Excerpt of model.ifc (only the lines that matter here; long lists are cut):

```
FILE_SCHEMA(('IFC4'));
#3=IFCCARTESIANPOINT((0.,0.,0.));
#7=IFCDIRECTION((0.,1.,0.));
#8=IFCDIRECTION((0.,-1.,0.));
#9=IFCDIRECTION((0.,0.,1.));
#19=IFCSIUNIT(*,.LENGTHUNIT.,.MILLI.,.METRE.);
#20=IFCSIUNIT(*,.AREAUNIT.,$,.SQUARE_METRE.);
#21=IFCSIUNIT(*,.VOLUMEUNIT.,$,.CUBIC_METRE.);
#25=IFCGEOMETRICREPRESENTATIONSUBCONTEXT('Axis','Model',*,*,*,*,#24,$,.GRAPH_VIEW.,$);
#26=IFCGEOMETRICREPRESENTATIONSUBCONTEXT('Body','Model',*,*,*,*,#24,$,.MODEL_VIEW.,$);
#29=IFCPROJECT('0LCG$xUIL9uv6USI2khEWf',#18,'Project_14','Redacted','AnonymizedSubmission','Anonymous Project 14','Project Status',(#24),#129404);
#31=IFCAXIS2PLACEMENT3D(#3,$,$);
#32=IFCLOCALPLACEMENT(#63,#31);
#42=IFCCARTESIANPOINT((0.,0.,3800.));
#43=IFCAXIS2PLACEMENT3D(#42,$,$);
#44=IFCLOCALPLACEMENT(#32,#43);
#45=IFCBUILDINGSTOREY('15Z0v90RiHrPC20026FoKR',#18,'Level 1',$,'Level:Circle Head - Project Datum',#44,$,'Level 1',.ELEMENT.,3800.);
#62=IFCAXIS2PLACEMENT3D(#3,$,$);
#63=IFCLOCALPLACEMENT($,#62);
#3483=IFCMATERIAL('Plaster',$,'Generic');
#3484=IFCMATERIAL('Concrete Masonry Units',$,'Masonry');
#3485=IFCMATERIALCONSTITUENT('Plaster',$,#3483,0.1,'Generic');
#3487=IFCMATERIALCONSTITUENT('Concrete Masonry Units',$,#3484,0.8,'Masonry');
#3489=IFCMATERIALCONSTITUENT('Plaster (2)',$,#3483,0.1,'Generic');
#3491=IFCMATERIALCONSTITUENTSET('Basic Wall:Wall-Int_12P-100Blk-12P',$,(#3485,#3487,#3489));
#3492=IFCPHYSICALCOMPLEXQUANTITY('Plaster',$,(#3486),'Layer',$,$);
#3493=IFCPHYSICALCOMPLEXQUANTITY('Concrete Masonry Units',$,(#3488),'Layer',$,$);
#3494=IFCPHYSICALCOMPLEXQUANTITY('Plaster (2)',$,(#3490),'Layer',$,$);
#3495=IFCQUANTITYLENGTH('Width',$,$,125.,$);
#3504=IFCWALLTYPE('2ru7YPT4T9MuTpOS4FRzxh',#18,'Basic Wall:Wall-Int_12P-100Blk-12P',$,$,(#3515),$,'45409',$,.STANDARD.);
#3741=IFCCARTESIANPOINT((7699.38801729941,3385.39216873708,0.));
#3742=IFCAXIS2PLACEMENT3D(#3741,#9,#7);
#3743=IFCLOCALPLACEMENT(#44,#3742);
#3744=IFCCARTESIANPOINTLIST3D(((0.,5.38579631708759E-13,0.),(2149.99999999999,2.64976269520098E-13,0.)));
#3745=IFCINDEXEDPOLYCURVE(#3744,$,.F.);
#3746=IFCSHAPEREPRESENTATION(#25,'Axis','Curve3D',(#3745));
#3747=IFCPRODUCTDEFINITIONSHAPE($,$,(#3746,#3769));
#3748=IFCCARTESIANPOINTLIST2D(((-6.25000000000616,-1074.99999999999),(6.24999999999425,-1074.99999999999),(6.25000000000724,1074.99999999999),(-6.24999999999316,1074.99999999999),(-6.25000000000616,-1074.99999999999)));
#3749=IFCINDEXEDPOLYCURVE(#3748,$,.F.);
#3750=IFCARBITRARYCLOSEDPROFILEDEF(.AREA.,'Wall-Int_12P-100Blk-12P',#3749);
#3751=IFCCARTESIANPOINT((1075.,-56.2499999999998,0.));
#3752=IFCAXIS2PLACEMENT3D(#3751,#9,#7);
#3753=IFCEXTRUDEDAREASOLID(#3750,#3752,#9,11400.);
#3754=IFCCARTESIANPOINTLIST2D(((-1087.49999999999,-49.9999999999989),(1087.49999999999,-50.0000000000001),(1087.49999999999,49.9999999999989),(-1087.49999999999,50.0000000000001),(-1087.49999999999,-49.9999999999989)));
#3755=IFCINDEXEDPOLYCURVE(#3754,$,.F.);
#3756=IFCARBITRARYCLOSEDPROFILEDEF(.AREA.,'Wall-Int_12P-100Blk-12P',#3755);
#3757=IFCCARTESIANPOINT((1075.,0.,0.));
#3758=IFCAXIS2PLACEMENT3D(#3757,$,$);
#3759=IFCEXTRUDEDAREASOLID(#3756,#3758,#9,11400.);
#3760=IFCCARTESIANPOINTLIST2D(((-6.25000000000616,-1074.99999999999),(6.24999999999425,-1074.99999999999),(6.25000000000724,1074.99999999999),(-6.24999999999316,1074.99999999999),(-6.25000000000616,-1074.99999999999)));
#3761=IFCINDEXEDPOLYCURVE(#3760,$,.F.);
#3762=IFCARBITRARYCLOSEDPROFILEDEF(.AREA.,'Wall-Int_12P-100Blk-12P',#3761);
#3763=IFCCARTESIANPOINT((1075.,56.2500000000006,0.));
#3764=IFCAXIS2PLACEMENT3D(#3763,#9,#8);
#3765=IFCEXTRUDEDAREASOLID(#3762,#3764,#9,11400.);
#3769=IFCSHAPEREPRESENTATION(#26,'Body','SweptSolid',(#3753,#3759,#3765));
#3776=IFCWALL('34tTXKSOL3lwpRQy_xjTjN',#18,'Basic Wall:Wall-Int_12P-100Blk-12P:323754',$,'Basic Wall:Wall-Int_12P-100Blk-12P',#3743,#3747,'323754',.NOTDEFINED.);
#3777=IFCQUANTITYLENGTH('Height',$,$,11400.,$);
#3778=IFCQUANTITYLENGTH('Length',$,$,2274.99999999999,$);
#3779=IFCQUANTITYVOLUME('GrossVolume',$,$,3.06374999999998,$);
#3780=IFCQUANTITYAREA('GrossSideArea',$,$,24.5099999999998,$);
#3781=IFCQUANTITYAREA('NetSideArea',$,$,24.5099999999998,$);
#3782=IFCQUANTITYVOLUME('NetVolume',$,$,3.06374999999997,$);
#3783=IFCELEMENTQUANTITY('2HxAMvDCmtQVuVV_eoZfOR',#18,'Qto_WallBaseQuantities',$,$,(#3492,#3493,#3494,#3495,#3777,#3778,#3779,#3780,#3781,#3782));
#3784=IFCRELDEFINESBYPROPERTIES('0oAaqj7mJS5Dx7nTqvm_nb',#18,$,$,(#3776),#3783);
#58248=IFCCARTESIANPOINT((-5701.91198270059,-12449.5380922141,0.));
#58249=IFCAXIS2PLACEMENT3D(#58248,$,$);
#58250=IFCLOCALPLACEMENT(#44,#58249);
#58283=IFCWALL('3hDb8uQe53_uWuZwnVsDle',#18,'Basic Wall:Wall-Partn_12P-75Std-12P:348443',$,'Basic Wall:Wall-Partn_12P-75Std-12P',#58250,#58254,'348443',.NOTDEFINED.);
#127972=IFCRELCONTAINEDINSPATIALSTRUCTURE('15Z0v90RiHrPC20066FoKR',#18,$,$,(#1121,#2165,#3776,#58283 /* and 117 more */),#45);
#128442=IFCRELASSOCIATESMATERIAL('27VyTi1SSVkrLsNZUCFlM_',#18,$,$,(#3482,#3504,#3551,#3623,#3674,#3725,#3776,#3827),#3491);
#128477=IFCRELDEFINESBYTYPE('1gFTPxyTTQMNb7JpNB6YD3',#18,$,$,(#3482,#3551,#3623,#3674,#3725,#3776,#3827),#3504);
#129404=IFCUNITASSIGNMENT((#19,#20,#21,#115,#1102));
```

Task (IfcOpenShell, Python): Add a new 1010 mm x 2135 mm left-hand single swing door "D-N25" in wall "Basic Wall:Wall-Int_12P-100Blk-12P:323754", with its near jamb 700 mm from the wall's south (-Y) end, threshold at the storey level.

```python
import numpy as np
import ifcopenshell
import ifcopenshell.api.feature
import ifcopenshell.api.geometry
import ifcopenshell.api.pset
import ifcopenshell.api.root
import ifcopenshell.api.spatial
import ifcopenshell.geom
import ifcopenshell.util.element
import ifcopenshell.util.placement
import ifcopenshell.util.representation
import ifcopenshell.util.shape
import ifcopenshell.util.unit

model = ifcopenshell.open("model.ifc")
unit_scale = ifcopenshell.util.unit.calculate_unit_scale(model)
area_scale = ifcopenshell.util.unit.calculate_unit_scale(model, "AREAUNIT")
volume_scale = ifcopenshell.util.unit.calculate_unit_scale(model, "VOLUMEUNIT")
settings = ifcopenshell.geom.settings()


def volume(element):
    """Net volume in cubic metres, openings subtracted."""
    shape = ifcopenshell.geom.create_shape(settings, element)
    return ifcopenshell.util.shape.get_volume(shape.geometry)


wall = model.by_guid("34tTXKSOL3lwpRQy_xjTjN")
storey = ifcopenshell.util.element.get_container(wall, ifc_class="IfcBuildingStorey")
context = ifcopenshell.util.representation.get_context(model, "Model", "Body", "MODEL_VIEW")
before = volume(wall)

width, height, from_end, sill = 1.01, 2.135, 0.7, 0.0  # metres

# The wall runs along its own X axis, and the end named is its -X end.
wall_shape = ifcopenshell.geom.create_shape(settings, wall)
x, y, z = ifcopenshell.util.shape.get_vertices(wall_shape.geometry).T
start = x.min() + from_end
face, thickness = float(y.min()), float(y.max() - y.min())
wall_matrix = ifcopenshell.util.placement.get_local_placement(wall.ObjectPlacement)
level = ifcopenshell.util.placement.get_local_placement(storey.ObjectPlacement)[2, 3]


def in_wall(x, y):
    """Placement at x, y metres in the wall's axes, at sill height."""
    matrix = wall_matrix.copy()
    matrix[:, 3] = wall_matrix @ np.array([x / unit_scale, y / unit_scale, 0.0, 1.0])
    matrix[2, 3] = level + sill / unit_scale
    return matrix


# Opening: a box that overshoots both wall faces by 50 mm.
opening = ifcopenshell.api.root.create_entity(model, ifc_class="IfcOpeningElement", predefined_type="OPENING")
box = ifcopenshell.api.geometry.add_wall_representation(
    model, context=context, length=width, height=height, thickness=thickness + 0.1
)
ifcopenshell.api.geometry.assign_representation(model, product=opening, representation=box)
ifcopenshell.api.geometry.edit_object_placement(model, product=opening, matrix=in_wall(start, face - 0.05), is_si=False)
ifcopenshell.api.feature.add_feature(model, feature=opening, element=wall)

door = ifcopenshell.api.root.create_entity(model, ifc_class="IfcDoor", name="D-N25", predefined_type="DOOR")
door.OverallWidth, door.OverallHeight = width / unit_scale, height / unit_scale
door.OperationType = "SINGLE_SWING_LEFT"
body = ifcopenshell.api.geometry.add_door_representation(
    model,
    context=context,
    overall_width=door.OverallWidth,
    overall_height=door.OverallHeight,
    operation_type="SINGLE_SWING_LEFT",
    lining_properties={"LiningDepth": thickness / unit_scale, "ThresholdDepth": thickness / unit_scale},
)
ifcopenshell.api.geometry.assign_representation(model, product=door, representation=body)
ifcopenshell.api.spatial.assign_container(model, products=[door], relating_structure=storey)
ifcopenshell.api.feature.add_filling(model, opening=opening, element=door)

# The lining spans the wall, so the door starts at the wall face.
ifcopenshell.api.geometry.edit_object_placement(model, product=door, matrix=in_wall(start, face), is_si=False)

after = volume(wall)

# Update the wall's stored quantities.
qto = model.by_id(ifcopenshell.util.element.get_pset(wall, "Qto_WallBaseQuantities", should_inherit=False)["id"])
ifcopenshell.api.pset.edit_qto(model, qto=qto, properties={
    "NetSideArea": after / thickness / area_scale,
    "NetVolume": after / volume_scale,
})

print(f"wall volume {before:.3f} -> {after:.3f} m3")

model.write("model_rev.ifc")
```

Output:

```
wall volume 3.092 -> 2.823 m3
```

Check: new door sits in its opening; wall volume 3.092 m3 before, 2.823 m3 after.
